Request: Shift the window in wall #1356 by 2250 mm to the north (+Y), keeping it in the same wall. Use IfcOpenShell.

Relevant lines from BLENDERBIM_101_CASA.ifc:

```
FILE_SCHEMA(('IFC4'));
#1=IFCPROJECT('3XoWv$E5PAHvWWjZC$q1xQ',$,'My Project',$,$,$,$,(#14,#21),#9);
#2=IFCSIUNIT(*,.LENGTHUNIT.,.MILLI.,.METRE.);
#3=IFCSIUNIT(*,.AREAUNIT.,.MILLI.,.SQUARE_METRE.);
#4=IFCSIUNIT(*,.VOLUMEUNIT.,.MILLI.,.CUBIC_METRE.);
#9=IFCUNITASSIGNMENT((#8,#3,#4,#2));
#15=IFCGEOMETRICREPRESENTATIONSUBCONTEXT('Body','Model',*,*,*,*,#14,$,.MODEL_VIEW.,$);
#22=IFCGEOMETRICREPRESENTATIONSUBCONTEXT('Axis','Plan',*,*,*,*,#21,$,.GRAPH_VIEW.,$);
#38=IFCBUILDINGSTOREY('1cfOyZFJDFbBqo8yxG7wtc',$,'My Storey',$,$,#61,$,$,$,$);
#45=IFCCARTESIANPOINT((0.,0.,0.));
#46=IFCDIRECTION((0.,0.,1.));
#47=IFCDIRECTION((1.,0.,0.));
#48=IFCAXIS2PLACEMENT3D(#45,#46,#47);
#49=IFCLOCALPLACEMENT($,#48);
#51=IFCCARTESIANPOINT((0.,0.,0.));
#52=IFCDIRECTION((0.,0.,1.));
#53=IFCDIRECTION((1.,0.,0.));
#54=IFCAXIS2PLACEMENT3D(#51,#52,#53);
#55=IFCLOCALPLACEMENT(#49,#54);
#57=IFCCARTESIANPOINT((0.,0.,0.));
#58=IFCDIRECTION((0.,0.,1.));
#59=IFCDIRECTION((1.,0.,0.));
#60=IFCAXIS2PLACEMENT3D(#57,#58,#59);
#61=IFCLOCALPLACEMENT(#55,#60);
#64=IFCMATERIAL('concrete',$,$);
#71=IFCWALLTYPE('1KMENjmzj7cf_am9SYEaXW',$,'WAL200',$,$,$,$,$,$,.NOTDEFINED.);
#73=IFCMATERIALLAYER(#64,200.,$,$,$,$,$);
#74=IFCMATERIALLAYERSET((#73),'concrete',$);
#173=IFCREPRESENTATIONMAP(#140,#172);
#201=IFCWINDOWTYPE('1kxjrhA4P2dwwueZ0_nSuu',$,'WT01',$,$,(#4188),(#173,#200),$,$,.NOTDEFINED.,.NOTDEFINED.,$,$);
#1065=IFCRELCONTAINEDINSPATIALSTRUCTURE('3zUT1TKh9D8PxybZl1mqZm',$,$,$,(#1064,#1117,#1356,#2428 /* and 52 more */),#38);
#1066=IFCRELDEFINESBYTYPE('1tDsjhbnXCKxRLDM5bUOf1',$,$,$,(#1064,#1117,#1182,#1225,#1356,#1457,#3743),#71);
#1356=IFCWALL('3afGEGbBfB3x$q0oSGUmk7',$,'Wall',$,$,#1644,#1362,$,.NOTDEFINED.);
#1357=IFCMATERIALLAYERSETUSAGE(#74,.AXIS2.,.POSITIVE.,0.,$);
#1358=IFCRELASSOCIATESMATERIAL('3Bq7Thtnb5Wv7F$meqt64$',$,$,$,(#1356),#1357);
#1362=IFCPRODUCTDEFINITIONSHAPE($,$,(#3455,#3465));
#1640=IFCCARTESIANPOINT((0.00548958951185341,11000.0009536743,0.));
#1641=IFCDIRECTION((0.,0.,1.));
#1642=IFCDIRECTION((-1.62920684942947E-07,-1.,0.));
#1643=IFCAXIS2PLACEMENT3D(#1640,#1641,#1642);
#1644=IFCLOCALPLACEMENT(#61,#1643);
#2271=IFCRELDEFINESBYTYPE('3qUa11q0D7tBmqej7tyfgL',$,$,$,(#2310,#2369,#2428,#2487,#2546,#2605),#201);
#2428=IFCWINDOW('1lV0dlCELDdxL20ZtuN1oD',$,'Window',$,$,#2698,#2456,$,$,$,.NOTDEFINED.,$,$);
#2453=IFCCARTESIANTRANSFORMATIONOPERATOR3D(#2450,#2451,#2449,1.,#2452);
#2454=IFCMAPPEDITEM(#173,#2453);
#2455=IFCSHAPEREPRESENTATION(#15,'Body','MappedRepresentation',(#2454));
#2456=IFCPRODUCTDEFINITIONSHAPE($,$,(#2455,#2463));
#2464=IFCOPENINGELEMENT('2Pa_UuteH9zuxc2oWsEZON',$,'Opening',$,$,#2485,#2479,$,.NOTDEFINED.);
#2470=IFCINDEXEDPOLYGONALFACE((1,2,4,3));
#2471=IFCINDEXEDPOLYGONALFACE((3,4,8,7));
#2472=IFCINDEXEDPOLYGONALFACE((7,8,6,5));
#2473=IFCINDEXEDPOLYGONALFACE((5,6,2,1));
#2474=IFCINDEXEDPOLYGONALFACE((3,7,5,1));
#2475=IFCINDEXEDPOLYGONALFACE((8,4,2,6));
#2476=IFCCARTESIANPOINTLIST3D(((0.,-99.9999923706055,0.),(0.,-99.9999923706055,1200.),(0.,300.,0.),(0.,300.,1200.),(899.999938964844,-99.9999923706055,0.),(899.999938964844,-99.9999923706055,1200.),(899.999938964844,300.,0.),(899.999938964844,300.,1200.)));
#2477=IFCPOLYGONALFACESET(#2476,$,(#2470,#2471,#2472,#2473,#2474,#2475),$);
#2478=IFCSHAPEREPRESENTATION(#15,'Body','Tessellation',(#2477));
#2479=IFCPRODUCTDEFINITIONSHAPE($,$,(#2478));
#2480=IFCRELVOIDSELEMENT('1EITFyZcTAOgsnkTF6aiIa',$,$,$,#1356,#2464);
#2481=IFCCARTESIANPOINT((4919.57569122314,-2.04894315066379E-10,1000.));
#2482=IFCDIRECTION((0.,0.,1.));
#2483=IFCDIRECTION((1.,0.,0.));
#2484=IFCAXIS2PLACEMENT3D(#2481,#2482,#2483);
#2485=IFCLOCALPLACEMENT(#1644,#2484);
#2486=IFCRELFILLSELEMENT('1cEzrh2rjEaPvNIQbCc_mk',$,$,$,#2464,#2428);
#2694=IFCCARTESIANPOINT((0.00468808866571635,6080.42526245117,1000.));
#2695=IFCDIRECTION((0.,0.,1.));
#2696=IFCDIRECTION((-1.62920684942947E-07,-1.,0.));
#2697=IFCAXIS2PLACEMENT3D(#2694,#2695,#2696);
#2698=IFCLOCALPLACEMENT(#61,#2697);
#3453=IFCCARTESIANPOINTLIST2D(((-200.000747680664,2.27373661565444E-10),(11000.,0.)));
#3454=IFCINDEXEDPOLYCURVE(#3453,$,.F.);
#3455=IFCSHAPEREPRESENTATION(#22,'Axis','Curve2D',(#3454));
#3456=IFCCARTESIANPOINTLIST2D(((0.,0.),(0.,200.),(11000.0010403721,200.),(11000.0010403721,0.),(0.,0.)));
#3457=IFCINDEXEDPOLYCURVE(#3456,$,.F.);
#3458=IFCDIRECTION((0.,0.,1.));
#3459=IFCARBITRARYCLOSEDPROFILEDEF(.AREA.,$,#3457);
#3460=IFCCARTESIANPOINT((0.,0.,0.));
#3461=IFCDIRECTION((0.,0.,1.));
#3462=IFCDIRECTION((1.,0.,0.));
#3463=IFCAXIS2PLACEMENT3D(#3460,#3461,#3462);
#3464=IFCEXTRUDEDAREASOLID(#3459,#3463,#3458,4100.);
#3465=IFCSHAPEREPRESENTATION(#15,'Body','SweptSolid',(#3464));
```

```python
import ifcopenshell
import ifcopenshell.api.geometry
import ifcopenshell.util.placement
import ifcopenshell.util.unit

model = ifcopenshell.open("BLENDERBIM_101_CASA.ifc")
unit_scale = ifcopenshell.util.unit.calculate_unit_scale(model)

window = model.by_id(2428)
opening = window.FillsVoids[0].RelatingOpeningElement
wall = opening.VoidsElements[0].RelatingBuildingElement

wall_matrix = ifcopenshell.util.placement.get_local_placement(wall.ObjectPlacement)
shift = wall_matrix[:3, 0] * -2.25 / unit_scale
before = ifcopenshell.util.placement.get_local_placement(window.ObjectPlacement)[:3, 3].copy()

# The window is not placed relative to its opening, so move both.
for product in (opening, window):
    matrix = ifcopenshell.util.placement.get_local_placement(product.ObjectPlacement)
    matrix[:3, 3] += shift
    ifcopenshell.api.geometry.edit_object_placement(model, product=product, matrix=matrix, is_si=False)

after = ifcopenshell.util.placement.get_local_placement(window.ObjectPlacement)[:3, 3]
print("window moved by", (after - before).round(3) + 0.0)

model.write("BLENDERBIM_101_CASA_v2.ifc")
```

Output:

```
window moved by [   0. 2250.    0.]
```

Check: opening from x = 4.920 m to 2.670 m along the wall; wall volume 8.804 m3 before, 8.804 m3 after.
